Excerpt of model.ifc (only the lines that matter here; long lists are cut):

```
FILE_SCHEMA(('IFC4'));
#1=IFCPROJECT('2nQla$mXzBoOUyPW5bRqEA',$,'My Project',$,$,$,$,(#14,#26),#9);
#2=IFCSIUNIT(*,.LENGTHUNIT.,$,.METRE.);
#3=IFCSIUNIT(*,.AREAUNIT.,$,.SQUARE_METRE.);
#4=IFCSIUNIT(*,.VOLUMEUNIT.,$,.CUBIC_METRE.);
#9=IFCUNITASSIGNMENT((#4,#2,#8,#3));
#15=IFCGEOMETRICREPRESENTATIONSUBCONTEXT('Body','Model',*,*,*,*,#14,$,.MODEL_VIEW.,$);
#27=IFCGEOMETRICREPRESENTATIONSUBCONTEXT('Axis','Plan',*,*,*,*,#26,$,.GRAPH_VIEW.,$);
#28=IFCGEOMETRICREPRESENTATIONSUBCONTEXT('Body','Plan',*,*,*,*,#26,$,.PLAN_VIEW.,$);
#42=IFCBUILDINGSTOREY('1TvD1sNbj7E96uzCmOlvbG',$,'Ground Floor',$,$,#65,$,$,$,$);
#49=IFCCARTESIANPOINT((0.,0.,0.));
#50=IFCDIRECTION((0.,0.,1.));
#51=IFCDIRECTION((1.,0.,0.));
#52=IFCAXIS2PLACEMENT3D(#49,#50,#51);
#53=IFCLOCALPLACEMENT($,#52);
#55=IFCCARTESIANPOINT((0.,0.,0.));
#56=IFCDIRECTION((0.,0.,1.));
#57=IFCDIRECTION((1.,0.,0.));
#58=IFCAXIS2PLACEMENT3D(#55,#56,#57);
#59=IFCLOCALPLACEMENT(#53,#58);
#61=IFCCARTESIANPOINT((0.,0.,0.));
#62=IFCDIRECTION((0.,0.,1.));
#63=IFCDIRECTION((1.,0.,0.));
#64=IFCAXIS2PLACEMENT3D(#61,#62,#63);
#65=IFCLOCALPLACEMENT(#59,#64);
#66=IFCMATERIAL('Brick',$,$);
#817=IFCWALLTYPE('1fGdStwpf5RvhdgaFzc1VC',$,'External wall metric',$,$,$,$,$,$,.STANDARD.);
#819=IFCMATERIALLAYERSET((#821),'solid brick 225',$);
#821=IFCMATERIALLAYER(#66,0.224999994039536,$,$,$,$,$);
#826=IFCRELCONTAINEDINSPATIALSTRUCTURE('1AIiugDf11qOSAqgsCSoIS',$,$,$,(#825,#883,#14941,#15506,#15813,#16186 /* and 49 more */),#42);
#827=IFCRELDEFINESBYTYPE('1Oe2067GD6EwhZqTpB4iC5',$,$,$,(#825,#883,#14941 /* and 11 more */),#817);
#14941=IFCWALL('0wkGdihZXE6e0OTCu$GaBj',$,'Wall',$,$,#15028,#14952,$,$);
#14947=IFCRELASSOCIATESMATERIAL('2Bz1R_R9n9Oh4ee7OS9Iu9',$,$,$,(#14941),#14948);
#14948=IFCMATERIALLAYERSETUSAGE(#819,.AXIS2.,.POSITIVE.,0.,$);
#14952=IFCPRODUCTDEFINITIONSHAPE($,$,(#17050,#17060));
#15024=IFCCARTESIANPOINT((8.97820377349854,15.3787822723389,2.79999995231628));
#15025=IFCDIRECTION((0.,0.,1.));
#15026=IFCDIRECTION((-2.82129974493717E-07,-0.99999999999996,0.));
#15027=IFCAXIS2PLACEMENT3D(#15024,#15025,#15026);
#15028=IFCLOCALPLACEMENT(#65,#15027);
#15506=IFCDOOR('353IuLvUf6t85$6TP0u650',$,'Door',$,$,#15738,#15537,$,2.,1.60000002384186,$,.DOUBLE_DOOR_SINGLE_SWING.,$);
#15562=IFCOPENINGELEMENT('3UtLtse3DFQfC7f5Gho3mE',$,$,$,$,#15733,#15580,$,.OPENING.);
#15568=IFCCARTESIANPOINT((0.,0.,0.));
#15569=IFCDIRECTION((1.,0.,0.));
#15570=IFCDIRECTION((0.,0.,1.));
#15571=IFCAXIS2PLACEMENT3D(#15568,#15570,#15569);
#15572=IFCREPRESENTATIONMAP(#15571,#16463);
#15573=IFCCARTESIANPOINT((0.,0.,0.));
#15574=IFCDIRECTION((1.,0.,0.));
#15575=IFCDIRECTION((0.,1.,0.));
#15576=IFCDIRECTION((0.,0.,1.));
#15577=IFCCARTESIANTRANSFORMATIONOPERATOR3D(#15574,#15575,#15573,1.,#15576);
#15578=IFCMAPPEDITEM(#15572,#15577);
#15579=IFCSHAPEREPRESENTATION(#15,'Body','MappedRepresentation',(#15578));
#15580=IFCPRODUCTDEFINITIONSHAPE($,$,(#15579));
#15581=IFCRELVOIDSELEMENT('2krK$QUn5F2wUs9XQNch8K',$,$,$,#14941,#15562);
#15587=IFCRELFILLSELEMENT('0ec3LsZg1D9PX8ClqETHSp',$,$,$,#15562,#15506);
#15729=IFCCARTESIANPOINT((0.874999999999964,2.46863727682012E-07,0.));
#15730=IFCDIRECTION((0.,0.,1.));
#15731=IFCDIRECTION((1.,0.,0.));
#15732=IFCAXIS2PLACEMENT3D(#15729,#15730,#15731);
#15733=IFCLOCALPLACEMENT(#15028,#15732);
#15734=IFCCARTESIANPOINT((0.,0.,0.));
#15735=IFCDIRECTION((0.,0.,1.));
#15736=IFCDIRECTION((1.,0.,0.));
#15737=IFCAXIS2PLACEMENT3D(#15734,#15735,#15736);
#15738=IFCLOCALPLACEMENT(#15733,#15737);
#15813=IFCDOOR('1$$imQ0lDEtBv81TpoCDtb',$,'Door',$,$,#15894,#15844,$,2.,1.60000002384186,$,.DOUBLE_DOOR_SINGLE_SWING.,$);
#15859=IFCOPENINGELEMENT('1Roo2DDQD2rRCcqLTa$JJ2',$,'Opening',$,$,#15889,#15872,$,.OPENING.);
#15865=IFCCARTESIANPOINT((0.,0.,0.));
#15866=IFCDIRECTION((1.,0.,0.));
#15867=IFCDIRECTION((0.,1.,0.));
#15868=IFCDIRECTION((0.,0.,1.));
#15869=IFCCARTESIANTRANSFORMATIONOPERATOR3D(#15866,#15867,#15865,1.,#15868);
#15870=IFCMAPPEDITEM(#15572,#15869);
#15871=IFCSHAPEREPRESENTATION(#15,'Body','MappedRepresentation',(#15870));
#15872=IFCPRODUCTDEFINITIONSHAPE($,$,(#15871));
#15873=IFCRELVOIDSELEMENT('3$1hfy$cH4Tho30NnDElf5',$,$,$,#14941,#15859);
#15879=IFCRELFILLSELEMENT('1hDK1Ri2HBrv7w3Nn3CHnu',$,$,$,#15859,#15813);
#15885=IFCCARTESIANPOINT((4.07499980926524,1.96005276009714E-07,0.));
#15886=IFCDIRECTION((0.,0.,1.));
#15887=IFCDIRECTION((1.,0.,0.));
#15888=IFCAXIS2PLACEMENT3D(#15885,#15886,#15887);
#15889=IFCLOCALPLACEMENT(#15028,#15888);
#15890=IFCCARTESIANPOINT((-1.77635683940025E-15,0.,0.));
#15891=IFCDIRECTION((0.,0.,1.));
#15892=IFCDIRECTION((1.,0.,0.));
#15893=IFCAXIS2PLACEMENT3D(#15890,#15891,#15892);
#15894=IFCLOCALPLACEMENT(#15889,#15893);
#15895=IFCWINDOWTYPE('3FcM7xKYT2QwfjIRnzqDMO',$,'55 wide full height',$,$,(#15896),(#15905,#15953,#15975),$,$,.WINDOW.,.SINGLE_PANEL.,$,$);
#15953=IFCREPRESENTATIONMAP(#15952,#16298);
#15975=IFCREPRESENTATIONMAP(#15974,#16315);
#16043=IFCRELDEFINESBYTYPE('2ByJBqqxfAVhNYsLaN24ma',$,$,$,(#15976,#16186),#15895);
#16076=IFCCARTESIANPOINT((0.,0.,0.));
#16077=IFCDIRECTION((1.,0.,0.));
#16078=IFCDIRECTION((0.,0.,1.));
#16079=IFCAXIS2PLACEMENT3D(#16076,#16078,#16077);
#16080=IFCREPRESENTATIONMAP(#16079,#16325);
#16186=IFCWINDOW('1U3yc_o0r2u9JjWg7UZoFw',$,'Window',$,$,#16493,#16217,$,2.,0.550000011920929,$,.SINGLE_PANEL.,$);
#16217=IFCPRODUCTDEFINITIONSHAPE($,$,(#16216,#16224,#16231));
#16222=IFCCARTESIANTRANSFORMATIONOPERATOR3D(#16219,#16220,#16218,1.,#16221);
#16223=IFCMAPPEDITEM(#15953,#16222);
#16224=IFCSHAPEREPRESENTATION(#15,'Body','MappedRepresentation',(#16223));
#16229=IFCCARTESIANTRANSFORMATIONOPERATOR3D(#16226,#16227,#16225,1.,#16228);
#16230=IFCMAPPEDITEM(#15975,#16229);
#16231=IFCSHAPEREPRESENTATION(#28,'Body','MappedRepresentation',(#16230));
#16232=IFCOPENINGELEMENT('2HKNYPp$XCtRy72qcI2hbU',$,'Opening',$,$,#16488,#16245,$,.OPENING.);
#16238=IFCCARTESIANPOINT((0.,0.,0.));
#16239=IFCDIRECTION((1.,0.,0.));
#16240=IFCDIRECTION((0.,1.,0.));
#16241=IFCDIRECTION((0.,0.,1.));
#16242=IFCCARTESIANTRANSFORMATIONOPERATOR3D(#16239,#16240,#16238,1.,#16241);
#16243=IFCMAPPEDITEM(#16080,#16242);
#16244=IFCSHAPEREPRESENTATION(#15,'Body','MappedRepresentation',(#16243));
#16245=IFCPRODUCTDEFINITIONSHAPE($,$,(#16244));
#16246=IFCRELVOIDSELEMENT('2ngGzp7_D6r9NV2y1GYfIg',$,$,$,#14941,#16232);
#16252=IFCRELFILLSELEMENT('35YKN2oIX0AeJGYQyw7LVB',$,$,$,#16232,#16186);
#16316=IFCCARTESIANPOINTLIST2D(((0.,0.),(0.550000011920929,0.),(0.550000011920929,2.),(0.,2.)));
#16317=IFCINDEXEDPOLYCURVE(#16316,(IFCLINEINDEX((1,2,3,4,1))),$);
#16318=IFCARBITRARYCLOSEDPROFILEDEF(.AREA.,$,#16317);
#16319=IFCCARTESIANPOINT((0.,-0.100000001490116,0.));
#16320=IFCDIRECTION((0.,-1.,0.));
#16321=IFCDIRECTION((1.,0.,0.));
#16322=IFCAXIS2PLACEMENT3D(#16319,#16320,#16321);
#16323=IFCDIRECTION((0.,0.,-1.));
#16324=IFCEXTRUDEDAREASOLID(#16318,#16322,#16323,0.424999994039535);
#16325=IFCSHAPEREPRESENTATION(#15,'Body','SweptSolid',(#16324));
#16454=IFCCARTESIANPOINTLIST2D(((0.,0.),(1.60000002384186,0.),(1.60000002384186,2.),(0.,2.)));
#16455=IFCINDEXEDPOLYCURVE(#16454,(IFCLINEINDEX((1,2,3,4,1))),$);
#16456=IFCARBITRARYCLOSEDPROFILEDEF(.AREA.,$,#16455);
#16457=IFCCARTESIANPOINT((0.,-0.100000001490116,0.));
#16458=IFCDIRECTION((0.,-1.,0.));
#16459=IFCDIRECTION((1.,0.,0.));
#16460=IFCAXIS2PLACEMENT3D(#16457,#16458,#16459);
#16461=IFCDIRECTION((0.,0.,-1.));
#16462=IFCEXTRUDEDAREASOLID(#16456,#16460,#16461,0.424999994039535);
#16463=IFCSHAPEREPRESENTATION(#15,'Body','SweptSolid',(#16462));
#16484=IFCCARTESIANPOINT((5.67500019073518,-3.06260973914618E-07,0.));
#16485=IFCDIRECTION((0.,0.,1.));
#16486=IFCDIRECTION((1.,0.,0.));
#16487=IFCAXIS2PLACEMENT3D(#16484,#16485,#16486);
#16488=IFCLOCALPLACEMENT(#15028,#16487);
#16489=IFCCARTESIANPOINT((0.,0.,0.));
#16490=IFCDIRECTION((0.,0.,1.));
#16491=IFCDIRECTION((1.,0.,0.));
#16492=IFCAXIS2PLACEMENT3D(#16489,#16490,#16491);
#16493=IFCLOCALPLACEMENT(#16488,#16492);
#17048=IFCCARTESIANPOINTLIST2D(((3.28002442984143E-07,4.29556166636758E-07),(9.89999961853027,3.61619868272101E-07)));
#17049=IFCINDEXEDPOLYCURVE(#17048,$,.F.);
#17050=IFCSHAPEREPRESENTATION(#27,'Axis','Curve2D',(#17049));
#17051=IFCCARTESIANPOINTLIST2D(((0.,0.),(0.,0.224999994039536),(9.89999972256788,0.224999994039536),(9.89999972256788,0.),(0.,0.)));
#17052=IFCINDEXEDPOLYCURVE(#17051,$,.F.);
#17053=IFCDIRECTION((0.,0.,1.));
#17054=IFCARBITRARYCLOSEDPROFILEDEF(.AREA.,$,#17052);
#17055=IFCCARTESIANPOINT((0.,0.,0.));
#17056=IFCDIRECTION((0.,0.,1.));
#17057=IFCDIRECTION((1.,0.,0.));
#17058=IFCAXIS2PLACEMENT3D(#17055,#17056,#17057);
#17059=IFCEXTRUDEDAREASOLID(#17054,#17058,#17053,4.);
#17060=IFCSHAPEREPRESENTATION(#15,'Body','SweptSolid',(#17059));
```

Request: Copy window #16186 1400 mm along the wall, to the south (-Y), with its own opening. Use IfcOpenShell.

```python
import ifcopenshell
import ifcopenshell.api.feature
import ifcopenshell.api.geometry
import ifcopenshell.api.root
import ifcopenshell.geom
import ifcopenshell.util.element
import ifcopenshell.util.placement
import ifcopenshell.util.shape
import ifcopenshell.util.unit

model = ifcopenshell.open("model.ifc")
unit_scale = ifcopenshell.util.unit.calculate_unit_scale(model)
settings = ifcopenshell.geom.settings()


def volume(element):
    """Net volume in cubic metres, openings subtracted."""
    shape = ifcopenshell.geom.create_shape(settings, element)
    return ifcopenshell.util.shape.get_volume(shape.geometry)


window = model.by_id(16186)
opening = window.FillsVoids[0].RelatingOpeningElement
wall = opening.VoidsElements[0].RelatingBuildingElement
before = volume(wall)
shift = ifcopenshell.util.placement.get_local_placement(wall.ObjectPlacement)[:3, 0] * 1.4 / unit_scale

# copy_class copies the void relationship, type, container and properties, but no geometry.
new_opening = ifcopenshell.api.root.copy_class(model, product=opening)
new_opening.Representation = ifcopenshell.util.element.copy_deep(
    model, opening.Representation, exclude=["IfcGeometricRepresentationContext", "IfcRepresentationMap"]
)
new_window = ifcopenshell.api.root.copy_class(model, product=window)
new_window.Representation = ifcopenshell.util.element.copy_deep(
    model, window.Representation, exclude=["IfcGeometricRepresentationContext", "IfcRepresentationMap"]
)
ifcopenshell.api.feature.add_filling(model, opening=new_opening, element=new_window)

for old, new in ((opening, new_opening), (window, new_window)):
    matrix = ifcopenshell.util.placement.get_local_placement(old.ObjectPlacement)
    matrix[:3, 3] += shift
    ifcopenshell.api.geometry.edit_object_placement(model, product=new, matrix=matrix, is_si=False)

after = volume(wall)

print(f"wall volume {before:.3f} -> {after:.3f} m3")

model.write("model_updated.ifc")
```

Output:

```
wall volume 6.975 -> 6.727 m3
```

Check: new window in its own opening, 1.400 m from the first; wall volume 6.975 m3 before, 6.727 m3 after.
